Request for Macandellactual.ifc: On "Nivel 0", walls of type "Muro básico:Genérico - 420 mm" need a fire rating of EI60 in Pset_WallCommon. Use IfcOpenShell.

First a look at what the model holds.

```python
import ifcopenshell
import ifcopenshell.util.element

model = ifcopenshell.open("Macandellactual.ifc")
print(model.schema)
storey = next(s for s in model.by_type("IfcBuildingStorey") if s.Name == "Nivel 0")
walls = [e for e in ifcopenshell.util.element.get_decomposition(storey) if e.is_a("IfcWall")]
seen = {}
for e in walls:
    element_type = ifcopenshell.util.element.get_type(e)
    key = (element_type.Name if element_type != e and element_type else None, ifcopenshell.util.element.get_pset(e, "Pset_WallCommon", "FireRating"))
    seen[key] = seen.get(key, 0) + 1
for (name, value), count in sorted(seen.items(), key=str):
    print(count, "x", name, "|", value)
```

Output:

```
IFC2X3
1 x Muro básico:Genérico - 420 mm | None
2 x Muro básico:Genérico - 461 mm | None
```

```python
import ifcopenshell
import ifcopenshell.api.pset
import ifcopenshell.util.element

model = ifcopenshell.open("Macandellactual.ifc")

storey = next(s for s in model.by_type("IfcBuildingStorey") if s.Name == "Nivel 0")
walls = [e for e in ifcopenshell.util.element.get_decomposition(storey) if e.is_a("IfcWall")]

count = 0
for e in walls:
    element_type = ifcopenshell.util.element.get_type(e)
    if element_type in (None, e) or element_type.Name != "Muro básico:Genérico - 420 mm":
        continue
    # add_pset returns the element's existing set when there is one.
    pset = ifcopenshell.api.pset.add_pset(model, product=e, name="Pset_WallCommon")
    ifcopenshell.api.pset.edit_pset(model, pset=pset, properties={"FireRating": "EI60"})
    count += 1

print(count, "walls updated")

model.write("Macandellactual_v2.ifc")
```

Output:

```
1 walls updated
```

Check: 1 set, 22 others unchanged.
